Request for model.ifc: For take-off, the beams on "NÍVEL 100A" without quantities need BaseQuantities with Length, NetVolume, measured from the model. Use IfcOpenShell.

First a look at what the model holds.

```python
import ifcopenshell
import ifcopenshell.util.element
import ifcopenshell.util.unit

model = ifcopenshell.open("model.ifc")
print(model.schema)
for unit_type in ("LENGTHUNIT", "AREAUNIT", "VOLUMEUNIT"):
    print(unit_type, ifcopenshell.util.unit.calculate_unit_scale(model, unit_type))
storey = next(s for s in model.by_type("IfcBuildingStorey") if s.Name == "NÍVEL 100A")
beams = [e for e in ifcopenshell.util.element.get_decomposition(storey) if e.is_a("IfcBeam")]
for e in sorted(beams, key=lambda e: e.id()):
    print(e.id(), e.is_a(), e.Name, list(ifcopenshell.util.element.get_psets(e, qtos_only=True)), sep=" | ")
```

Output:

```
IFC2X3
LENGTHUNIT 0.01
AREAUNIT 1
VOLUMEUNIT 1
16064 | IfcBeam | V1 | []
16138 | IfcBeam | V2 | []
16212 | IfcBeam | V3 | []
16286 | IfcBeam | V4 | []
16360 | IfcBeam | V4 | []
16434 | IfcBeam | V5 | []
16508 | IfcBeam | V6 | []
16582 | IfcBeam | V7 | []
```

```python
import ifcopenshell
import ifcopenshell.api.pset
import ifcopenshell.geom
import ifcopenshell.util.element
import ifcopenshell.util.shape
import ifcopenshell.util.unit

model = ifcopenshell.open("model.ifc")
unit_scale = ifcopenshell.util.unit.calculate_unit_scale(model)
volume_scale = ifcopenshell.util.unit.calculate_unit_scale(model, "VOLUMEUNIT")
settings = ifcopenshell.geom.settings()

storey = next(s for s in model.by_type("IfcBuildingStorey") if s.Name == "NÍVEL 100A")
beams = [e for e in ifcopenshell.util.element.get_decomposition(storey) if e.is_a("IfcBeam")]

for e in sorted(beams, key=lambda e: e.id()):
    if ifcopenshell.util.element.get_psets(e, qtos_only=True, should_inherit=False):
        continue
    # Geometry comes back in metres, in the element's own axes.
    shape = ifcopenshell.geom.create_shape(settings, e)
    values = {
        "Length": ifcopenshell.util.shape.get_max_xyz(shape.geometry) / unit_scale,
        "NetVolume": ifcopenshell.util.shape.get_volume(shape.geometry) / volume_scale,
    }
    qto = ifcopenshell.api.pset.add_qto(model, product=e, name="BaseQuantities")
    ifcopenshell.api.pset.edit_qto(model, qto=qto, properties=values)
    print(e.id(), {k: round(v, 3) for k, v in values.items()})

model.write("model_edited.ifc")
```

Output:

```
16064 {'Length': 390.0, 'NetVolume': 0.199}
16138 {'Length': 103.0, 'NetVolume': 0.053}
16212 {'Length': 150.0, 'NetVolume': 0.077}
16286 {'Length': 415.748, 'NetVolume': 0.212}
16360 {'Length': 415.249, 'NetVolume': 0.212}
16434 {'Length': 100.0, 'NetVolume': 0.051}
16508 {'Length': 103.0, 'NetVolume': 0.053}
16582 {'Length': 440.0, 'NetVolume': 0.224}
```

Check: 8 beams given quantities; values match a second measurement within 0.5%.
